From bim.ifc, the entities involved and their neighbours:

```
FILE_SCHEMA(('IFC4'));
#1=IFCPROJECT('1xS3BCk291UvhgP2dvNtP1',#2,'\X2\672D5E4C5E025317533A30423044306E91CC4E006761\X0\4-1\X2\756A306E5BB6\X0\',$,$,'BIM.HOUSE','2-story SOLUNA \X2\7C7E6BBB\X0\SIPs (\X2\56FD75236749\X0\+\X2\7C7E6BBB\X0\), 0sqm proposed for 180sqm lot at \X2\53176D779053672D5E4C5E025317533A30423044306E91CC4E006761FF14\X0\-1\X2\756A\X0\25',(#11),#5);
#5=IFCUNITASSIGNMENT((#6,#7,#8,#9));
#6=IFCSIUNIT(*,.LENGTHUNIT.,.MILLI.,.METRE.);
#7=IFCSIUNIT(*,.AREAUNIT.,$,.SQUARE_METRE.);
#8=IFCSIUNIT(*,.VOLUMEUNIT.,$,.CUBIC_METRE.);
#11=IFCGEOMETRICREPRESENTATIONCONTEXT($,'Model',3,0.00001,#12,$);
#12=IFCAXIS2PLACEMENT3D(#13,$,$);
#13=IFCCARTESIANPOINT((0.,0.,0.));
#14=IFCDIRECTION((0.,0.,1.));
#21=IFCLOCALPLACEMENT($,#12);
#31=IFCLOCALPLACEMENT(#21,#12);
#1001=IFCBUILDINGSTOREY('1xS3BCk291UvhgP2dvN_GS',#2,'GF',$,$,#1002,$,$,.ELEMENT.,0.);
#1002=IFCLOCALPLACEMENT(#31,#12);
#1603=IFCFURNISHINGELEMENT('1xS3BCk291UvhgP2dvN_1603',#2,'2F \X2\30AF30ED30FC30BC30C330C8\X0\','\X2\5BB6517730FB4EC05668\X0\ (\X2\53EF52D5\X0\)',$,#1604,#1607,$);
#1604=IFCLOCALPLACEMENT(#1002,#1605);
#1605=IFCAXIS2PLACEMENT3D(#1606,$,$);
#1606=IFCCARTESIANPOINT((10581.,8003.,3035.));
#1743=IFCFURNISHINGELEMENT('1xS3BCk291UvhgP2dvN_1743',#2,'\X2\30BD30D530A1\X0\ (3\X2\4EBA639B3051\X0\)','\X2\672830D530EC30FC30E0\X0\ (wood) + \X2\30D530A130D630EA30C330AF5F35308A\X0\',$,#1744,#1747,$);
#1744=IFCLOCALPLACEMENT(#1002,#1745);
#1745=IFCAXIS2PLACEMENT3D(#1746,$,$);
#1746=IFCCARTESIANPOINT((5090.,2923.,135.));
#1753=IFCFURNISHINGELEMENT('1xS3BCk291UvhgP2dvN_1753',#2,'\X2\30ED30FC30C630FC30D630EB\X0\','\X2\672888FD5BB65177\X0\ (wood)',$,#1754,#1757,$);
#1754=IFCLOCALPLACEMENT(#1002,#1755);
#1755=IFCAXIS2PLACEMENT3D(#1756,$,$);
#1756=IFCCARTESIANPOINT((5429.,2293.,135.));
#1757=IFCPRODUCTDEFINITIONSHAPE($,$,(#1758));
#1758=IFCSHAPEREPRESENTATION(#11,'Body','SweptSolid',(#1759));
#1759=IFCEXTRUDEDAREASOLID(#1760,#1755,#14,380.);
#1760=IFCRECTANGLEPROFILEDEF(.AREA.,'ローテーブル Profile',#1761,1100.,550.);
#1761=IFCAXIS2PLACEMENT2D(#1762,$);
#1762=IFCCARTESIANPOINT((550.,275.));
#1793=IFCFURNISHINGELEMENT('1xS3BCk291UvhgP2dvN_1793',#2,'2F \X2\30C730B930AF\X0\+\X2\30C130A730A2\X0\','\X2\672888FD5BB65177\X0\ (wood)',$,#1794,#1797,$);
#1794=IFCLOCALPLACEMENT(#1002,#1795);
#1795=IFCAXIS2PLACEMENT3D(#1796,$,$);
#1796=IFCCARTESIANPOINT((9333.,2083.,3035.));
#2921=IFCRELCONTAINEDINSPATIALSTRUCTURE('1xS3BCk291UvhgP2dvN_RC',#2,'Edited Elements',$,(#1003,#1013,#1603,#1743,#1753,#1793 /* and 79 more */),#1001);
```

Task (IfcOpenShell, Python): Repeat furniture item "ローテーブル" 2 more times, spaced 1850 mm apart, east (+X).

```python
import numpy as np
import ifcopenshell
import ifcopenshell.api.geometry
import ifcopenshell.api.root
import ifcopenshell.util.element
import ifcopenshell.util.placement
import ifcopenshell.util.unit

model = ifcopenshell.open("bim.ifc")
unit_scale = ifcopenshell.util.unit.calculate_unit_scale(model)


def reuse_history(source, copy):
    """copy_class also copies each property set's owner history, people and application; keep the originals."""
    for rel in copy.IsDefinedBy:
        if rel.is_a("IfcRelDefinesByProperties") and (history := rel.RelatingPropertyDefinition.OwnerHistory):
            rel.RelatingPropertyDefinition.OwnerHistory = source.OwnerHistory
            ifcopenshell.util.element.remove_deep2(model, history)


source = model.by_guid("1xS3BCk291UvhgP2dvN_1753")
base = ifcopenshell.util.placement.get_local_placement(source.ObjectPlacement)
step = np.array([1.0, 0.0, 0.0]) * 1.85 / unit_scale

for i in range(1, 3):
    copy = ifcopenshell.api.root.copy_class(model, product=source)
    copy.Representation = ifcopenshell.util.element.copy_deep(
        model, source.Representation, exclude=["IfcGeometricRepresentationContext", "IfcRepresentationMap"]
    )
    reuse_history(source, copy)
    matrix = base.copy()
    matrix[:3, 3] += i * step
    print("added at", matrix[:3, 3].round(3) + 0.0)
    ifcopenshell.api.geometry.edit_object_placement(model, product=copy, matrix=matrix, is_si=False)

model.write("bim_v2.ifc")
```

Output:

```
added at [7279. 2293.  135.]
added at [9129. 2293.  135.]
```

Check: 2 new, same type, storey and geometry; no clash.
